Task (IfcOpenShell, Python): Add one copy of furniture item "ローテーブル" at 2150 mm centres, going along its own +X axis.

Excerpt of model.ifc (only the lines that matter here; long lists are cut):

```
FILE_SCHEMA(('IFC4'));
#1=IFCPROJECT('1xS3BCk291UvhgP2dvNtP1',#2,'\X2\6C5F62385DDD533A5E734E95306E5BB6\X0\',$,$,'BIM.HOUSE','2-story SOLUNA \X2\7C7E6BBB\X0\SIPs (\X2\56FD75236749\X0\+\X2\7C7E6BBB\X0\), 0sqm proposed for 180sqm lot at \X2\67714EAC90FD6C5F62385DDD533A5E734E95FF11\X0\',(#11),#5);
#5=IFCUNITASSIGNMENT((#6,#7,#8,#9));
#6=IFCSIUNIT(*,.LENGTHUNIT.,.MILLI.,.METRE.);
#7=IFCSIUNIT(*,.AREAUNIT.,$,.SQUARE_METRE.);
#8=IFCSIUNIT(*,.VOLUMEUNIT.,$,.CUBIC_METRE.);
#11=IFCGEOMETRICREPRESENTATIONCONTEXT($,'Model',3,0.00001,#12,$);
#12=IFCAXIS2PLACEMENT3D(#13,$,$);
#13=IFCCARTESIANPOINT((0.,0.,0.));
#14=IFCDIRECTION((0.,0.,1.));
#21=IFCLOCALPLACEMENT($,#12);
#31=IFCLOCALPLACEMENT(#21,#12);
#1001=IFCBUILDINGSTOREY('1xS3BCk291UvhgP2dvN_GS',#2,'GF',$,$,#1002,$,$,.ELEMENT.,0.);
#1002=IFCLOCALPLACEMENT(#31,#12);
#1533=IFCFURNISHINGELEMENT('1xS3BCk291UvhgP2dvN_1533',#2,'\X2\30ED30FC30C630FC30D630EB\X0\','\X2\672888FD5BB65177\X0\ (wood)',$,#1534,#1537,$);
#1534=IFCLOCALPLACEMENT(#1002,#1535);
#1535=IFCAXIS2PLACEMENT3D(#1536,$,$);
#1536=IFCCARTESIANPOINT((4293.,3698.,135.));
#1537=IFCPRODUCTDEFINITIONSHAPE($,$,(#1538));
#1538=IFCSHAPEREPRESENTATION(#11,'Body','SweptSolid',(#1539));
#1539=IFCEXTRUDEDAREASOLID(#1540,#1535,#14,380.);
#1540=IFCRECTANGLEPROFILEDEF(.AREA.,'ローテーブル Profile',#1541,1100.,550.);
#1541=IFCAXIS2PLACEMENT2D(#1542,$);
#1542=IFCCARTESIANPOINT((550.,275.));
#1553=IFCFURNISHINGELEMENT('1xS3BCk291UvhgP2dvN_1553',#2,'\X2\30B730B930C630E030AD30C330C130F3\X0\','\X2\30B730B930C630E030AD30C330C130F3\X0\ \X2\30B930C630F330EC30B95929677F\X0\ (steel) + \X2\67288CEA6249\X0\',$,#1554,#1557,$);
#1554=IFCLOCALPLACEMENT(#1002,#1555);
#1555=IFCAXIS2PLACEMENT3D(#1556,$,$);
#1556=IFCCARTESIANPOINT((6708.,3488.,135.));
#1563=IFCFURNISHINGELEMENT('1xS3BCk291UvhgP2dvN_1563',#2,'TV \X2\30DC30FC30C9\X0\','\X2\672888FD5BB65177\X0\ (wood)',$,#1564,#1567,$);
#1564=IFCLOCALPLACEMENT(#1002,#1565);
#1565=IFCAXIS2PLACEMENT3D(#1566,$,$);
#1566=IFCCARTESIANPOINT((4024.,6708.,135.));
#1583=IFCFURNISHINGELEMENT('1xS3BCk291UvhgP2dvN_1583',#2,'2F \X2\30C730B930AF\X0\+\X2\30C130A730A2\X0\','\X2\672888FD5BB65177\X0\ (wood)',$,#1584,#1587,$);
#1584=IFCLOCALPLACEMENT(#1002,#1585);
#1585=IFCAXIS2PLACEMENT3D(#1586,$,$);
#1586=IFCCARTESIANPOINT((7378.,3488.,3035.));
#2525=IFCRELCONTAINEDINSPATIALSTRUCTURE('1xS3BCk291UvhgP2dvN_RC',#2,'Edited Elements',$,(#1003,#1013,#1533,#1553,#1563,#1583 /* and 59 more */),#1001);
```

```python
import ifcopenshell
import ifcopenshell.api.geometry
import ifcopenshell.api.root
import ifcopenshell.util.element
import ifcopenshell.util.placement
import ifcopenshell.util.unit

model = ifcopenshell.open("model.ifc")
unit_scale = ifcopenshell.util.unit.calculate_unit_scale(model)


def reuse_history(source, copy):
    """copy_class also copies each property set's owner history, people and application; keep the originals."""
    for rel in copy.IsDefinedBy:
        if rel.is_a("IfcRelDefinesByProperties") and (history := rel.RelatingPropertyDefinition.OwnerHistory):
            rel.RelatingPropertyDefinition.OwnerHistory = source.OwnerHistory
            ifcopenshell.util.element.remove_deep2(model, history)


source = model.by_guid("1xS3BCk291UvhgP2dvN_1533")
base = ifcopenshell.util.placement.get_local_placement(source.ObjectPlacement)
step = base[:3, 0] * 2.15 / unit_scale

for i in range(1, 2):
    copy = ifcopenshell.api.root.copy_class(model, product=source)
    copy.Representation = ifcopenshell.util.element.copy_deep(
        model, source.Representation, exclude=["IfcGeometricRepresentationContext", "IfcRepresentationMap"]
    )
    reuse_history(source, copy)
    matrix = base.copy()
    matrix[:3, 3] += i * step
    print("added at", matrix[:3, 3].round(3) + 0.0)
    ifcopenshell.api.geometry.edit_object_placement(model, product=copy, matrix=matrix, is_si=False)

model.write("model_edited.ifc")
```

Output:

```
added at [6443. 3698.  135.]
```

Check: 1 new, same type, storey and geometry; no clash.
